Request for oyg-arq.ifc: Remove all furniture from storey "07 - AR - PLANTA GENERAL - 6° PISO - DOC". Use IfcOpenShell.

First a look at what the model holds.

```python
import ifcopenshell
import ifcopenshell.util.element

model = ifcopenshell.open("oyg-arq.ifc")
print(model.schema)
storey = next(s for s in model.by_type("IfcBuildingStorey") if s.Name == "07 - AR - PLANTA GENERAL - 6° PISO - DOC")
furniture = [e for e in ifcopenshell.util.element.get_decomposition(storey) if e.is_a("IfcFurnishingElement")]
seen = {}
for e in furniture:
    element_type = ifcopenshell.util.element.get_type(e)
    name = element_type.Name if element_type not in (None, e) else None
    seen[name] = seen.get(name, 0) + 1
for name, count in sorted(seen.items(), key=str):
    print(count, "x", name)
```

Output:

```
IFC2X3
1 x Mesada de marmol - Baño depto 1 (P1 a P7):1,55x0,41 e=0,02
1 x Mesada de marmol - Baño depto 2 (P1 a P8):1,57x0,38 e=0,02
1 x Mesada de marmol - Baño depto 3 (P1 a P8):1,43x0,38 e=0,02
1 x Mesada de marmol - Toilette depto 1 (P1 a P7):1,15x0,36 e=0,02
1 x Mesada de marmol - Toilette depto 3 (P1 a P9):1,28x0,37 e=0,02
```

```python
import ifcopenshell
import ifcopenshell.api.root
import ifcopenshell.util.element

model = ifcopenshell.open("oyg-arq.ifc")

storey = next(s for s in model.by_type("IfcBuildingStorey") if s.Name == "07 - AR - PLANTA GENERAL - 6° PISO - DOC")
furniture = [e for e in ifcopenshell.util.element.get_decomposition(storey) if e.is_a("IfcFurnishingElement")]

for e in furniture:
    ifcopenshell.api.root.remove_product(model, product=e)
print(len(furniture), "removed")

model.write("oyg-arq_rev.ifc")
```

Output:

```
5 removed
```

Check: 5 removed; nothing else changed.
